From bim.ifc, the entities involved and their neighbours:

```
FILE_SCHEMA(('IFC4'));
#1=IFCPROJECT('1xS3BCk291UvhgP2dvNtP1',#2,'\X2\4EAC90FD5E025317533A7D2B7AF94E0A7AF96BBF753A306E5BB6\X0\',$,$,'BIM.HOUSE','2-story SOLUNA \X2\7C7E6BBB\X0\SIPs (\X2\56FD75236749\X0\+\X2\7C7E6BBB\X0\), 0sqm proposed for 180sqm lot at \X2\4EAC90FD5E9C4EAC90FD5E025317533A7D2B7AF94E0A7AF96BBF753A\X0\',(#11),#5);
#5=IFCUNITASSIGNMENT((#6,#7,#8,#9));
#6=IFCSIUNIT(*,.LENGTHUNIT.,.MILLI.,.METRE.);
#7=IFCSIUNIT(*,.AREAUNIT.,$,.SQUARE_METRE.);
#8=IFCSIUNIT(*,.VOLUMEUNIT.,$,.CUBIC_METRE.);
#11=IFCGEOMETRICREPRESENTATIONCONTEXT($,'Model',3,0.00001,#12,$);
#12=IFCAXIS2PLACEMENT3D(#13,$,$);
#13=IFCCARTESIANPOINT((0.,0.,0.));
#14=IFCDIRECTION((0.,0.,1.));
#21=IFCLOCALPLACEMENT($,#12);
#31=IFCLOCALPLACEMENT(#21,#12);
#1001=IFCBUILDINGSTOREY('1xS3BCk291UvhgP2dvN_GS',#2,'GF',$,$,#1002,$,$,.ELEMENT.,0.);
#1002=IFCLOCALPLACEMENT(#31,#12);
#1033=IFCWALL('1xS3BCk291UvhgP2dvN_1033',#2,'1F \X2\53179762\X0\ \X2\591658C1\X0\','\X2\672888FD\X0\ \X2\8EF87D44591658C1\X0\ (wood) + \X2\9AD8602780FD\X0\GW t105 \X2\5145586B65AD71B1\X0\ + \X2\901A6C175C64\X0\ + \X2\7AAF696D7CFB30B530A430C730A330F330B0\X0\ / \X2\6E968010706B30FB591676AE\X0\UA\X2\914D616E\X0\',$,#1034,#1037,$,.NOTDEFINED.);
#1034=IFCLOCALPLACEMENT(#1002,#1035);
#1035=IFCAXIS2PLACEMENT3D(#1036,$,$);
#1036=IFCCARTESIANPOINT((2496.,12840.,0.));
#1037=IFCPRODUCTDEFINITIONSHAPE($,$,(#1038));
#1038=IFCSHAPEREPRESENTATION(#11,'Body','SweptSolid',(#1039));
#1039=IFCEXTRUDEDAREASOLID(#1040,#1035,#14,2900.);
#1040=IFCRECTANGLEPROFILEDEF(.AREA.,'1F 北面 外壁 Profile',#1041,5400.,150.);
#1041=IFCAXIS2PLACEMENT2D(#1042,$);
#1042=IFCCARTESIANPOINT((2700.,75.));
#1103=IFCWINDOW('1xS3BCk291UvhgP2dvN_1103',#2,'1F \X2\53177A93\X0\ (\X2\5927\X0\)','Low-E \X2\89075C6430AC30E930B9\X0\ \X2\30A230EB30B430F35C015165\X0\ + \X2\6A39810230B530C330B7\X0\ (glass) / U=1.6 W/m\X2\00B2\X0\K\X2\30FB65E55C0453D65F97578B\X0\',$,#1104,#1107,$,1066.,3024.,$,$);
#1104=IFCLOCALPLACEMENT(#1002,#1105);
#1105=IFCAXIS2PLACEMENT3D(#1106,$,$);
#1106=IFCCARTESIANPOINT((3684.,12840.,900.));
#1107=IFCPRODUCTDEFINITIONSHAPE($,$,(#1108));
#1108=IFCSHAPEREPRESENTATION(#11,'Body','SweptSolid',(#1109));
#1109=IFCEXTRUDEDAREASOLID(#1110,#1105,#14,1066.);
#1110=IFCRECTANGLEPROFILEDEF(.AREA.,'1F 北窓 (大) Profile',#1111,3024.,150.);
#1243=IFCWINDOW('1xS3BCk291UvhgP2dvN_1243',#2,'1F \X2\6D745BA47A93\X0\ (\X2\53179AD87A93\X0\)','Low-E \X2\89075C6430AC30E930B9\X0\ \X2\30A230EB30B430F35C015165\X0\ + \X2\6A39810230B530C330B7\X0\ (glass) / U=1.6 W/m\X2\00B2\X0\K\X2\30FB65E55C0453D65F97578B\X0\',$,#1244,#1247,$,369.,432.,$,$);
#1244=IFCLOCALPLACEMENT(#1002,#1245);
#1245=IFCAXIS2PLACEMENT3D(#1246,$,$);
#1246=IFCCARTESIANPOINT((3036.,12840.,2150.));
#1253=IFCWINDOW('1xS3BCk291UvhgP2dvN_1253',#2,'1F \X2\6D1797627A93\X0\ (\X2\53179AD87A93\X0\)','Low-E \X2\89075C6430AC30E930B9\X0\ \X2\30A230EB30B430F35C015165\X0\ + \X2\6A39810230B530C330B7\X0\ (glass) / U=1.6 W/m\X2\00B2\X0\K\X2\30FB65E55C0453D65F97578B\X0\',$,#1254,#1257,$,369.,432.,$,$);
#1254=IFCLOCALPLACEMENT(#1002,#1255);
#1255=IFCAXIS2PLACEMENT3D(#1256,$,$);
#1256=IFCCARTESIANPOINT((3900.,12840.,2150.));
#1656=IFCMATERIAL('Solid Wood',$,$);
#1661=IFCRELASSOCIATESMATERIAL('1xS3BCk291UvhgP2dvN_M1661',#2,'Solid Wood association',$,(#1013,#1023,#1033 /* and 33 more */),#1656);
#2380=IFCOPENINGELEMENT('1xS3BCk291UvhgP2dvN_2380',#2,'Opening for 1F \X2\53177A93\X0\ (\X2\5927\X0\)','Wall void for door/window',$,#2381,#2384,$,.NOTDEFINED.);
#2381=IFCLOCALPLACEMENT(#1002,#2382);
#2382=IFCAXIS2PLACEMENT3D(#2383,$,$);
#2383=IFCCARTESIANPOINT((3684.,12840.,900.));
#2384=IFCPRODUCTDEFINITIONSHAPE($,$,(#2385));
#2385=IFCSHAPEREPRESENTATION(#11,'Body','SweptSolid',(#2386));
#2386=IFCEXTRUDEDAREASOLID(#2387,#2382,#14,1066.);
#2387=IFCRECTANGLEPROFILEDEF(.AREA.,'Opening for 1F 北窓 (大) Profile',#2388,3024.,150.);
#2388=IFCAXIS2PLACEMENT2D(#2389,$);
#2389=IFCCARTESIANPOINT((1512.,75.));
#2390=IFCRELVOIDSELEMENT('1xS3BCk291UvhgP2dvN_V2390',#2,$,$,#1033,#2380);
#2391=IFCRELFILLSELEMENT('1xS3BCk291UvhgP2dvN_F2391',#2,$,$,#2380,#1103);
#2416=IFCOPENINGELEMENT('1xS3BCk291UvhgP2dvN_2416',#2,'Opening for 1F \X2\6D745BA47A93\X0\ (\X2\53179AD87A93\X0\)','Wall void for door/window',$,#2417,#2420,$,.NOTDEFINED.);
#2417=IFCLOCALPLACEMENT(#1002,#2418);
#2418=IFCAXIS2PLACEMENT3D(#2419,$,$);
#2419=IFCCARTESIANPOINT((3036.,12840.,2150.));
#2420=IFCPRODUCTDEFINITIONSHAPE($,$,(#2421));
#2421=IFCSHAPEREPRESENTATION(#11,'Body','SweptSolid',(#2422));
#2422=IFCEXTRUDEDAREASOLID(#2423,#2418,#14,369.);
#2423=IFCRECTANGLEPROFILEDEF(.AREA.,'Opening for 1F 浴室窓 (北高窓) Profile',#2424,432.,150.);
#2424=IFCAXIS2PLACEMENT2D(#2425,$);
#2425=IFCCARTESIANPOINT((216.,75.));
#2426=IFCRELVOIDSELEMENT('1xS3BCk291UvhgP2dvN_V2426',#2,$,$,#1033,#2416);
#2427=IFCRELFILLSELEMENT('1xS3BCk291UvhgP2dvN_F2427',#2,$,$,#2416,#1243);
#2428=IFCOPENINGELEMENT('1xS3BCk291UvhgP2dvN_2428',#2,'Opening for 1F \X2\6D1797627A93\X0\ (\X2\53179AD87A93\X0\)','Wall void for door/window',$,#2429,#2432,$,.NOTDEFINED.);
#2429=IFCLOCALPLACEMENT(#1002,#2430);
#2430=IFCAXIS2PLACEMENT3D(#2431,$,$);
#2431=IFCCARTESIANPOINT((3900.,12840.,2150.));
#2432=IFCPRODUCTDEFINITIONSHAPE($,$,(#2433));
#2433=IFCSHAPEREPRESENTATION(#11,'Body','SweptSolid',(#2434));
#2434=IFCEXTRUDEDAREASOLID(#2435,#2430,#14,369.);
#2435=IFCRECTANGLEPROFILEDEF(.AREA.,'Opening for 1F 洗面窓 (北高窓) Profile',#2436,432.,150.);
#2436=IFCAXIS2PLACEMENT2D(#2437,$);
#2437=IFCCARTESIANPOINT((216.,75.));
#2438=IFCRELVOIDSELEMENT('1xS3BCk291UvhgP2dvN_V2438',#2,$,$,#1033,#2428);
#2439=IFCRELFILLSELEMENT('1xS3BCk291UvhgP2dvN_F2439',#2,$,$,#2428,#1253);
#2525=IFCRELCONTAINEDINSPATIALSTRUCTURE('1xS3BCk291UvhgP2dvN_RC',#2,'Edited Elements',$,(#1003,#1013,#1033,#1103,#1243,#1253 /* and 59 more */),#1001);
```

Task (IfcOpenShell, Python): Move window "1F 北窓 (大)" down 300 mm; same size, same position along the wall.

```python
import numpy as np
import ifcopenshell
import ifcopenshell.api.geometry
import ifcopenshell.util.placement
import ifcopenshell.util.unit

model = ifcopenshell.open("bim.ifc")
unit_scale = ifcopenshell.util.unit.calculate_unit_scale(model)

window = model.by_guid("1xS3BCk291UvhgP2dvN_1103")
opening = window.FillsVoids[0].RelatingOpeningElement
dz = -300.0

shift = np.array([0.0, 0.0, dz])
# The window is not placed relative to its opening, so move both.
for product in (opening, window):
    matrix = ifcopenshell.util.placement.get_local_placement(product.ObjectPlacement)
    matrix[:3, 3] += shift
    ifcopenshell.api.geometry.edit_object_placement(model, product=product, matrix=matrix, is_si=False)

print(f"moved by {dz * unit_scale:+.3f} m")

model.write("bim-out.ifc")
```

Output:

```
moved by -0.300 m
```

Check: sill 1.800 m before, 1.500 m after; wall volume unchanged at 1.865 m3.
